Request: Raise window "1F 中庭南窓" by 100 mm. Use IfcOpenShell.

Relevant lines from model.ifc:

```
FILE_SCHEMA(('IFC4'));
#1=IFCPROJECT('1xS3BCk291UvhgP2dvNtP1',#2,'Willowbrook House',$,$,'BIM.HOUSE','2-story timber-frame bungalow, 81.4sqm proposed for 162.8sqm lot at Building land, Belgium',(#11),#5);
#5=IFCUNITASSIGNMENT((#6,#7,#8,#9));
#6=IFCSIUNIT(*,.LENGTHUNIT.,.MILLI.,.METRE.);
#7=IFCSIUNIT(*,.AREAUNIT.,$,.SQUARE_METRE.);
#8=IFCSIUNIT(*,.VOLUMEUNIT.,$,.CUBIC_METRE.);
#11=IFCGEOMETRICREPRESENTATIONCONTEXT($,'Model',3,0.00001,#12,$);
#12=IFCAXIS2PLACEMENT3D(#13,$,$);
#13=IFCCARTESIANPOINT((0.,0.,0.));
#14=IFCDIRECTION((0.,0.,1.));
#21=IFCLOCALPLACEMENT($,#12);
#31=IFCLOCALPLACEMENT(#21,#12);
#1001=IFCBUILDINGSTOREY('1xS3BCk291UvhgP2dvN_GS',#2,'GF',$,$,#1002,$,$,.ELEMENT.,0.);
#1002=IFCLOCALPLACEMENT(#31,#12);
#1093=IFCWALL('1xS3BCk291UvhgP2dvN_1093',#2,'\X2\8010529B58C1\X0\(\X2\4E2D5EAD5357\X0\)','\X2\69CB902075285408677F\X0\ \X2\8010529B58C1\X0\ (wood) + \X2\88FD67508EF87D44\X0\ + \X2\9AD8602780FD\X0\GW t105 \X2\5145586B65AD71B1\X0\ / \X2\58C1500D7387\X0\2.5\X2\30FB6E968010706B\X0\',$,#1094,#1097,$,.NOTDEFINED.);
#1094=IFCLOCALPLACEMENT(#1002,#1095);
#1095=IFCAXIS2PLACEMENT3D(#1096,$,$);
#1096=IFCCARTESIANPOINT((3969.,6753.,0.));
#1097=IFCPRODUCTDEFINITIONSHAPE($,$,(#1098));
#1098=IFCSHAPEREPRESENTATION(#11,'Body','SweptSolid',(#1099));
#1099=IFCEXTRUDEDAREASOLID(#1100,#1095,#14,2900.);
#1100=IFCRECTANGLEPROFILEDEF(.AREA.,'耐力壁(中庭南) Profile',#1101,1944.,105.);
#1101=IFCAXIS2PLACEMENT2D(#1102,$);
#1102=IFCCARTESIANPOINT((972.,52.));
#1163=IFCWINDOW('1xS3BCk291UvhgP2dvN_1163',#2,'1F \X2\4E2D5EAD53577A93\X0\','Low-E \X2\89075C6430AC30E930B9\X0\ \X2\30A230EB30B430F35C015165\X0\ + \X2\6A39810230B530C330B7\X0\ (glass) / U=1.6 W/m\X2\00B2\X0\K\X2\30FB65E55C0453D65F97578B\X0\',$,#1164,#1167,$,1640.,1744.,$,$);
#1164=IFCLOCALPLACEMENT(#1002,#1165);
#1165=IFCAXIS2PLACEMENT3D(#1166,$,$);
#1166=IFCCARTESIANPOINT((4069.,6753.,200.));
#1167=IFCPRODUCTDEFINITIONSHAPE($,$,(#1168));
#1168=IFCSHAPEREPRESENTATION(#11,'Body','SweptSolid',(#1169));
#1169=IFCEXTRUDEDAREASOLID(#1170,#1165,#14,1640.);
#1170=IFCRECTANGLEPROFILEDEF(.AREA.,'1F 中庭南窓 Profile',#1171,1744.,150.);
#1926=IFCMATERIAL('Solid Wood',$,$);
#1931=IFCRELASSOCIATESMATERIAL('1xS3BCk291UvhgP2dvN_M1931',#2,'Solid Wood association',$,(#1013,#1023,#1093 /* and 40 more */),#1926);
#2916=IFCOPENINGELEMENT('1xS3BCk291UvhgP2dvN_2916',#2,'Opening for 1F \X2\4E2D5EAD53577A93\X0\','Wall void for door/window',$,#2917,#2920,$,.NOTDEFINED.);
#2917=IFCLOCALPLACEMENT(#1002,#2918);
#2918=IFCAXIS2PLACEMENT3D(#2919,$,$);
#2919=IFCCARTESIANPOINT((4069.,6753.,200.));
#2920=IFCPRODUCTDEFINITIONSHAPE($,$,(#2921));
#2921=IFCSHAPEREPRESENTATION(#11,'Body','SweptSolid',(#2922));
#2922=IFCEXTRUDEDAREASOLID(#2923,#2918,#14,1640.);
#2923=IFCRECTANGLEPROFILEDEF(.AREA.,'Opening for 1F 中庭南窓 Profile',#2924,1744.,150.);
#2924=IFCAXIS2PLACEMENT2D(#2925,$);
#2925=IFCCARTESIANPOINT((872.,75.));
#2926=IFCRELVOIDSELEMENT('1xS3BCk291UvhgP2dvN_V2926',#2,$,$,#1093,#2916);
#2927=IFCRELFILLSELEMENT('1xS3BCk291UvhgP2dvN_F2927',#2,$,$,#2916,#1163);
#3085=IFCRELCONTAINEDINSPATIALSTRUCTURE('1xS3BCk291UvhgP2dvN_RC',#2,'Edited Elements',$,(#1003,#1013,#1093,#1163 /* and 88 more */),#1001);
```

```python
import numpy as np
import ifcopenshell
import ifcopenshell.api.geometry
import ifcopenshell.util.placement
import ifcopenshell.util.unit

model = ifcopenshell.open("model.ifc")
unit_scale = ifcopenshell.util.unit.calculate_unit_scale(model)

window = model.by_guid("1xS3BCk291UvhgP2dvN_1163")
opening = window.FillsVoids[0].RelatingOpeningElement
dz = 0.1 / unit_scale

shift = np.array([0.0, 0.0, dz])
# The window is not placed relative to its opening, so move both.
for product in (opening, window):
    matrix = ifcopenshell.util.placement.get_local_placement(product.ObjectPlacement)
    matrix[:3, 3] += shift
    ifcopenshell.api.geometry.edit_object_placement(model, product=product, matrix=matrix, is_si=False)

print(f"moved by {dz * unit_scale:+.3f} m")

model.write("model-out.ifc")
```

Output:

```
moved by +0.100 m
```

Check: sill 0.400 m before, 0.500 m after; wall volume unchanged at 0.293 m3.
